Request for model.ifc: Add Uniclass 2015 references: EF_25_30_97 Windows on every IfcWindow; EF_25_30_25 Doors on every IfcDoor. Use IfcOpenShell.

First a look at what the model holds.

```python
import ifcopenshell

model = ifcopenshell.open("model.ifc")
print(model.schema)
print("classifications:", [c.Name for c in model.by_type("IfcClassification")])
for ifc_class in ("IfcDoor", "IfcRoof", "IfcStair", "IfcWall", "IfcWindow"):
    print(ifc_class, len(model.by_type(ifc_class)))
```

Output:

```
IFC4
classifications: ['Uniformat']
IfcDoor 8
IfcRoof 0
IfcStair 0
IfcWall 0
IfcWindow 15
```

```python
import ifcopenshell
import ifcopenshell.api.classification

model = ifcopenshell.open("model.ifc")

system = ifcopenshell.api.classification.add_classification(model, classification="Uniclass 2015")

codes = {
    "IfcWindow": ("EF_25_30_97", "Windows"),
    "IfcDoor": ("EF_25_30_25", "Doors"),
}
for ifc_class, (code, name) in codes.items():
    products = model.by_type(ifc_class)
    ifcopenshell.api.classification.add_reference(
        model, products=products, classification=system, identification=code, name=name
    )
    print(code, len(products))

model.write("model-out.ifc")
```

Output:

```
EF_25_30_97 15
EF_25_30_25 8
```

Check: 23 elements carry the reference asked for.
